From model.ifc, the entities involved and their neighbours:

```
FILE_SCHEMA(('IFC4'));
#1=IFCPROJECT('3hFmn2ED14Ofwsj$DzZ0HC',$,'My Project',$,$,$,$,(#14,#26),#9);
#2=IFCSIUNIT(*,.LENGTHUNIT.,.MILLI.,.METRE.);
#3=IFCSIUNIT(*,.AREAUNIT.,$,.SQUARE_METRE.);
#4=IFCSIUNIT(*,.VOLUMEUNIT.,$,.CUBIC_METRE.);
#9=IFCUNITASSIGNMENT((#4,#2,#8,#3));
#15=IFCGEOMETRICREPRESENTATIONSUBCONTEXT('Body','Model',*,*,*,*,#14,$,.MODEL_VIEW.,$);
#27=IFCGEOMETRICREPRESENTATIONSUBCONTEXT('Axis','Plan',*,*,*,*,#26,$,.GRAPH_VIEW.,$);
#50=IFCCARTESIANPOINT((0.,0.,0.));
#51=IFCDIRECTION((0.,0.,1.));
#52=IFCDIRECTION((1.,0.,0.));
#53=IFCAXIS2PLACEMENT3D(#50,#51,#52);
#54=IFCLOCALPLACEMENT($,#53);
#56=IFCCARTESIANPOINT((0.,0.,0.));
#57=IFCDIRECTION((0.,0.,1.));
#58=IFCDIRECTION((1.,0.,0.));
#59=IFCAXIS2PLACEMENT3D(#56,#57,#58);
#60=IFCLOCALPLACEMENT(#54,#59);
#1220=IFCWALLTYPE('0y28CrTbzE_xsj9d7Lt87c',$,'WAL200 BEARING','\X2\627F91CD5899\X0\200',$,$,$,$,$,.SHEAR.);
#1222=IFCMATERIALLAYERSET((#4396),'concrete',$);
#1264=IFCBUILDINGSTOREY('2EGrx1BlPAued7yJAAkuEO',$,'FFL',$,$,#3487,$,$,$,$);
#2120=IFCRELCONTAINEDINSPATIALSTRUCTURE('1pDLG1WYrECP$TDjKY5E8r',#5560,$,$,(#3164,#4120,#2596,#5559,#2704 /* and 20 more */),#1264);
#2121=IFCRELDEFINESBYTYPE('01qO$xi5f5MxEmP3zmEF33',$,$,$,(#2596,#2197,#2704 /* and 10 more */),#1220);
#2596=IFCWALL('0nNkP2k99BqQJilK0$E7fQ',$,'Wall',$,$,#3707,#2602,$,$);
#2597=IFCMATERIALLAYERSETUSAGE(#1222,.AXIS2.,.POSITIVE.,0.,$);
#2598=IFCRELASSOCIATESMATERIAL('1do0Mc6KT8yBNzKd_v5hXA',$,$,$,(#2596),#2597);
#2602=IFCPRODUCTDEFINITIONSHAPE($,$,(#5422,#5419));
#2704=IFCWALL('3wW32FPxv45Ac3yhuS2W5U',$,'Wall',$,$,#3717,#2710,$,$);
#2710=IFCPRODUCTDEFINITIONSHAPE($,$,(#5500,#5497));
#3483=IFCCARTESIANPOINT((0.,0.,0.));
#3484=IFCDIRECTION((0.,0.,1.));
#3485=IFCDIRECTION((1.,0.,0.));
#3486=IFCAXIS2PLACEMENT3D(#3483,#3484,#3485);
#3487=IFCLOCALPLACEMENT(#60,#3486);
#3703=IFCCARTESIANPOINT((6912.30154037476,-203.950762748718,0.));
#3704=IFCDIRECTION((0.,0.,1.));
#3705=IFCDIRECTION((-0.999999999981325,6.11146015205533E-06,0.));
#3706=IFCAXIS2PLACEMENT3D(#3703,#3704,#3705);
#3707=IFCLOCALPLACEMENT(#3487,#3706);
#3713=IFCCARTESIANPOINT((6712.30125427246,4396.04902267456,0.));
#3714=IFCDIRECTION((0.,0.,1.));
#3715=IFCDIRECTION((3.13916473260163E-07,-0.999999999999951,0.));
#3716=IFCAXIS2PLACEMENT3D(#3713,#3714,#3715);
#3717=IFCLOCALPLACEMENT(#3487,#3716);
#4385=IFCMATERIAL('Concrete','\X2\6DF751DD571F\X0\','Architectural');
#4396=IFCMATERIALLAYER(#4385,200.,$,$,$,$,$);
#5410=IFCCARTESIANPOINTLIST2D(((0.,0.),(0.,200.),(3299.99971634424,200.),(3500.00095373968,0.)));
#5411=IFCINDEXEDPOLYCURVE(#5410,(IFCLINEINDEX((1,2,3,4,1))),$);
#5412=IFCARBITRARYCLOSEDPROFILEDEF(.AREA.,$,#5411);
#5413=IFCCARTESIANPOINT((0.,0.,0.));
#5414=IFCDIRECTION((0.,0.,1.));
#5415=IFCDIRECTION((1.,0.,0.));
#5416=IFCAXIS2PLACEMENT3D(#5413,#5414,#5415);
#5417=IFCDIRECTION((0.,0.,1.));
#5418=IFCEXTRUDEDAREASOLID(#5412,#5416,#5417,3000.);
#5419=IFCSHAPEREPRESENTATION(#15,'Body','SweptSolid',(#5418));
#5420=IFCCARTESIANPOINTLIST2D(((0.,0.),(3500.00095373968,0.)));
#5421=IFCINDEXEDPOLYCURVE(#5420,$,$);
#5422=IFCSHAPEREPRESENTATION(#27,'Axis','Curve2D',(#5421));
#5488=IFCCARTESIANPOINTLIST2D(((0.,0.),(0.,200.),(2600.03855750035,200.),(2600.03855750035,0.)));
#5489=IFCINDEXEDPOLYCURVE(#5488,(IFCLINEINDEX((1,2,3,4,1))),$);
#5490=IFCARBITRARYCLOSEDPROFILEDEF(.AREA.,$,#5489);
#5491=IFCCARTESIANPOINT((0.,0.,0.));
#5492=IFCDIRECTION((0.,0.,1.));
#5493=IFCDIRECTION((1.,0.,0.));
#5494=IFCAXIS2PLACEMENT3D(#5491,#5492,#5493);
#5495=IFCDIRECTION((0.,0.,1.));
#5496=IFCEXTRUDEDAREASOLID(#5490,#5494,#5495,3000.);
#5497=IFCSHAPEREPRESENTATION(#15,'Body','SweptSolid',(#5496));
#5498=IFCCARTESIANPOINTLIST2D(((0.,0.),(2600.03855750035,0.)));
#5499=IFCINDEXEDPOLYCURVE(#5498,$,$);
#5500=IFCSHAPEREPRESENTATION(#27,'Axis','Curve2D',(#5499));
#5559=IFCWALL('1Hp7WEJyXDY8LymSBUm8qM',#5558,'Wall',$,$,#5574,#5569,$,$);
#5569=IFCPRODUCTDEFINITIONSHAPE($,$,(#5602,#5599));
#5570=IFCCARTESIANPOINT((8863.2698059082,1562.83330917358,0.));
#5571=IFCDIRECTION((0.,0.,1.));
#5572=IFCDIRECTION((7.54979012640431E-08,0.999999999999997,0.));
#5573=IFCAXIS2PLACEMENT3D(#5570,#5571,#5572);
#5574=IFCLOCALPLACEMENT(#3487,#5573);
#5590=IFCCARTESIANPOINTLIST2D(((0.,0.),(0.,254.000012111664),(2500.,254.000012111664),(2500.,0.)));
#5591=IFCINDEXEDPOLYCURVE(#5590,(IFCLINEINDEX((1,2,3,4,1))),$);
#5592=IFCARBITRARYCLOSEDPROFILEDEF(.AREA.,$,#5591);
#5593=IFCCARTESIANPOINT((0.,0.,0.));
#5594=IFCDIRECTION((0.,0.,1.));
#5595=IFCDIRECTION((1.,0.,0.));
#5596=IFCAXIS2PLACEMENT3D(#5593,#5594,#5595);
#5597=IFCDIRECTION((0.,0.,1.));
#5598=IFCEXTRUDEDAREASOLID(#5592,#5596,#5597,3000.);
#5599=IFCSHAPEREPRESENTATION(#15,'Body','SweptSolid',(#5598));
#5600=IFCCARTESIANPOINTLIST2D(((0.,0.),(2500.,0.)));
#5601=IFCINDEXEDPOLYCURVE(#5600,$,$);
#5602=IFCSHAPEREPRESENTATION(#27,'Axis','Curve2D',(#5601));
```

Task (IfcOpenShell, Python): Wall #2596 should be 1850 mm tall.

```python
import ifcopenshell
import ifcopenshell.geom
import ifcopenshell.util.representation
import ifcopenshell.util.shape

model = ifcopenshell.open("model.ifc")
settings = ifcopenshell.geom.settings()


def volume(element):
    """Net volume in cubic metres, openings subtracted."""
    shape = ifcopenshell.geom.create_shape(settings, element)
    return ifcopenshell.util.shape.get_volume(shape.geometry)


wall = model.by_id(2596)
before = volume(wall)

body = ifcopenshell.util.representation.get_representation(wall, "Model", "Body")
solid = body.Items[0]
old_height = solid.Depth
solid.Depth = 1850.0
after = volume(wall)

print(f"height {old_height:g} -> {solid.Depth:g}, volume {before:.3f} -> {after:.3f} m3")

model.write("model_updated.ifc")
```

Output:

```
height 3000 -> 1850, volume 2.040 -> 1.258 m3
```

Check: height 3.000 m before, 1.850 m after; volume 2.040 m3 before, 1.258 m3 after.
